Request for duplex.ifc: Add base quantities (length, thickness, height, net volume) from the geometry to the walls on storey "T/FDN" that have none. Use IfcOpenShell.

First a look at what the model holds.

```python
import ifcopenshell
import ifcopenshell.util.element
import ifcopenshell.util.unit

model = ifcopenshell.open("duplex.ifc")
print(model.schema)
for unit_type in ("LENGTHUNIT", "AREAUNIT", "VOLUMEUNIT"):
    print(unit_type, ifcopenshell.util.unit.calculate_unit_scale(model, unit_type))
storey = next(s for s in model.by_type("IfcBuildingStorey") if s.Name == "T/FDN")
walls = [e for e in ifcopenshell.util.element.get_decomposition(storey) if e.is_a("IfcWall")]
for e in sorted(walls, key=lambda e: e.id()):
    print(e.id(), e.is_a(), e.Name, list(ifcopenshell.util.element.get_psets(e, qtos_only=True)), sep=" | ")
```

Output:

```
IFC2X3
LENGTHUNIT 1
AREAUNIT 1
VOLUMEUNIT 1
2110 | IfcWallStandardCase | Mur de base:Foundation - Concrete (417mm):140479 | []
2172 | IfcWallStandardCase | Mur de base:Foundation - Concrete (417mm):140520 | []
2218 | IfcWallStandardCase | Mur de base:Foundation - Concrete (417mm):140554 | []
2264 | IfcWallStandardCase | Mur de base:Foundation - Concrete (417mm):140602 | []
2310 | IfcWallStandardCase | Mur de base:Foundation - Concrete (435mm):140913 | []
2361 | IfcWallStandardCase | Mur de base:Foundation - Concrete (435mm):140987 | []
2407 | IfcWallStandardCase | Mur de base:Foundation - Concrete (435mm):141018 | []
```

```python
import ifcopenshell
import ifcopenshell.api.pset
import ifcopenshell.geom
import ifcopenshell.util.element
import ifcopenshell.util.shape
import ifcopenshell.util.unit

model = ifcopenshell.open("duplex.ifc")
unit_scale = ifcopenshell.util.unit.calculate_unit_scale(model)
volume_scale = ifcopenshell.util.unit.calculate_unit_scale(model, "VOLUMEUNIT")
settings = ifcopenshell.geom.settings()

storey = next(s for s in model.by_type("IfcBuildingStorey") if s.Name == "T/FDN")
walls = [e for e in ifcopenshell.util.element.get_decomposition(storey) if e.is_a("IfcWall")]

for e in sorted(walls, key=lambda e: e.id()):
    if ifcopenshell.util.element.get_psets(e, qtos_only=True, should_inherit=False):
        continue
    # Geometry comes back in metres, in the element's own axes.
    shape = ifcopenshell.geom.create_shape(settings, e)
    values = {
        "Length": ifcopenshell.util.shape.get_x(shape.geometry) / unit_scale,
        "Width": ifcopenshell.util.shape.get_y(shape.geometry) / unit_scale,
        "Height": ifcopenshell.util.shape.get_z(shape.geometry) / unit_scale,
        "NetVolume": ifcopenshell.util.shape.get_volume(shape.geometry) / volume_scale,
    }
    qto = ifcopenshell.api.pset.add_qto(model, product=e, name="BaseQuantities")
    ifcopenshell.api.pset.edit_qto(model, qto=qto, properties=values)
    print(e.id(), {k: round(v, 3) for k, v in values.items()})

model.write("duplex_rev.ifc")
```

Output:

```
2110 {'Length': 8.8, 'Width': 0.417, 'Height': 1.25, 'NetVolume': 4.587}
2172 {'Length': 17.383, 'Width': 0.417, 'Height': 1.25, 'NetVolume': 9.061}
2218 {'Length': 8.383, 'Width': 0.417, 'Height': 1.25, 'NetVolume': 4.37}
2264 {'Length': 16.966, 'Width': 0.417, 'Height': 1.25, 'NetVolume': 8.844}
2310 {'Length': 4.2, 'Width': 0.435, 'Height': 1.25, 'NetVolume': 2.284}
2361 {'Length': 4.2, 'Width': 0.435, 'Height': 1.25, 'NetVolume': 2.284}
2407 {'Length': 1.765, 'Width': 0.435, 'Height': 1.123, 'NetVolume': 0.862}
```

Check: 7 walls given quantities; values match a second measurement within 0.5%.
